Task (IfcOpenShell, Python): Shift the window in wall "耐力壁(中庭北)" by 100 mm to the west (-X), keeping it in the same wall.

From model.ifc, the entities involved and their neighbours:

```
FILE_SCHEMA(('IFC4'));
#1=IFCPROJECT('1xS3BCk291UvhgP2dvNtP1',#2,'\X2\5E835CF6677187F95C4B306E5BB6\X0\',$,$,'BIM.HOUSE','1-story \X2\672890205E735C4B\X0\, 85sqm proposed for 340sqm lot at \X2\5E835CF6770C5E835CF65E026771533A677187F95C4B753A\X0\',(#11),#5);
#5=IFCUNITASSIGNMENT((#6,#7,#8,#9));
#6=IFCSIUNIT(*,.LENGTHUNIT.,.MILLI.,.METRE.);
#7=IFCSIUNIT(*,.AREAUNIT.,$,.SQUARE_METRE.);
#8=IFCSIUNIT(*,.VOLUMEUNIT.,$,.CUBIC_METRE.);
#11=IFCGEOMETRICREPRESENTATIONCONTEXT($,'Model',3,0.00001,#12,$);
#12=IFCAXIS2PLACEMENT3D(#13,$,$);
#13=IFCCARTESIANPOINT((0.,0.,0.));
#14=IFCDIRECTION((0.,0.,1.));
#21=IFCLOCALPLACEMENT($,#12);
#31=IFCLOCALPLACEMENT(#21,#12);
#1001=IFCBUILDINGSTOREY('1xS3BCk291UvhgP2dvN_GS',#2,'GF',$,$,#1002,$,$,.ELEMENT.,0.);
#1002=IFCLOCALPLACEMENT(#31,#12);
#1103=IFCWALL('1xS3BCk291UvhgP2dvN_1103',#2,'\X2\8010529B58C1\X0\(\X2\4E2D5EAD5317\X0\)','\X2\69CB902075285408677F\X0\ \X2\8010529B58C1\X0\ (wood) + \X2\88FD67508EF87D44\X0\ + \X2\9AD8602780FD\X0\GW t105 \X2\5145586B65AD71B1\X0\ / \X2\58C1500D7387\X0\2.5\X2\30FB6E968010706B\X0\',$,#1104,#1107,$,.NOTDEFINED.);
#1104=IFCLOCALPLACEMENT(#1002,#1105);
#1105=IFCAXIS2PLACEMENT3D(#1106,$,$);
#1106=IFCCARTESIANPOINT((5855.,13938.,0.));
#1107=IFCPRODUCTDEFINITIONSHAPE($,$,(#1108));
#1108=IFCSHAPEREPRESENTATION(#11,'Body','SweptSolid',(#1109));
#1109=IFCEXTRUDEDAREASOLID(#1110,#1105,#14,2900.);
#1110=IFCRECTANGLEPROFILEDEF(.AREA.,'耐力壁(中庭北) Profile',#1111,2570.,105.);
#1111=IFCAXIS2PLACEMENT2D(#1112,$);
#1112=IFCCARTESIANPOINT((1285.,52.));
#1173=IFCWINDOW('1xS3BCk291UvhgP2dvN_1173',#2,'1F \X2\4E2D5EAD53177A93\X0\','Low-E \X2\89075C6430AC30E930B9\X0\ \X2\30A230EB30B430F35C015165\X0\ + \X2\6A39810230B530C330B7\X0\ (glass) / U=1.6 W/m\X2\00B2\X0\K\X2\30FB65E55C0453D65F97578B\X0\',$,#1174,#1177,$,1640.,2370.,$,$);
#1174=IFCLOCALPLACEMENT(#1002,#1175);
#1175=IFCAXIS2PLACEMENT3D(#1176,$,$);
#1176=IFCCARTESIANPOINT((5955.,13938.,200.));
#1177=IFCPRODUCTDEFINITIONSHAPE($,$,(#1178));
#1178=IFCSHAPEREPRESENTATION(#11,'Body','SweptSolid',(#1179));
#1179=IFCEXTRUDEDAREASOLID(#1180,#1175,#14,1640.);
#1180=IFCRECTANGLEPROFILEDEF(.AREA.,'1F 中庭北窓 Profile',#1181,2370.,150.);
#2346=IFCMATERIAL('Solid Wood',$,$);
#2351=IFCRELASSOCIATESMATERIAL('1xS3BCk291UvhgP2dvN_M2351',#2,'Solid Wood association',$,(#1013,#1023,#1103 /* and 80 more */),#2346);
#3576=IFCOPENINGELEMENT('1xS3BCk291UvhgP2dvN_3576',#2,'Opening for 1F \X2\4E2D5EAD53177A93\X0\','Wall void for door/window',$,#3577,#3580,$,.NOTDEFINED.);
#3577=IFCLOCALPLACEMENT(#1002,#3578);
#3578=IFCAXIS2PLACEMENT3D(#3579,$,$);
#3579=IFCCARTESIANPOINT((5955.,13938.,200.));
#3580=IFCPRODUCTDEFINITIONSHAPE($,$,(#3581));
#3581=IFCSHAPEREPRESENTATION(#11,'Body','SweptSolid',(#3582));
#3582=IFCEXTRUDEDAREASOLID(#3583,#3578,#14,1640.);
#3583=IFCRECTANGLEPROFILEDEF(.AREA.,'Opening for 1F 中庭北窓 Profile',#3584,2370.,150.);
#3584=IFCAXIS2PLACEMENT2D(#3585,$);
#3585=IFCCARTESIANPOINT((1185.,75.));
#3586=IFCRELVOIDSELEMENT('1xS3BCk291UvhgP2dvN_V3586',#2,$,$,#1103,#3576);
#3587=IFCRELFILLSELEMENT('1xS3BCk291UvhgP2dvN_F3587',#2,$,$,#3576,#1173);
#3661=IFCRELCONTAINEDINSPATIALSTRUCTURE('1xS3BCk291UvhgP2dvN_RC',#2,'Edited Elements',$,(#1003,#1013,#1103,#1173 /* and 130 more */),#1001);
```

```python
import ifcopenshell
import ifcopenshell.api.geometry
import ifcopenshell.util.placement

model = ifcopenshell.open("model.ifc")

window = model.by_guid("1xS3BCk291UvhgP2dvN_1173")
opening = window.FillsVoids[0].RelatingOpeningElement
wall = opening.VoidsElements[0].RelatingBuildingElement

wall_matrix = ifcopenshell.util.placement.get_local_placement(wall.ObjectPlacement)
shift = wall_matrix[:3, 0] * -100.0
before = ifcopenshell.util.placement.get_local_placement(window.ObjectPlacement)[:3, 3].copy()

# The window is not placed relative to its opening, so move both.
for product in (opening, window):
    matrix = ifcopenshell.util.placement.get_local_placement(product.ObjectPlacement)
    matrix[:3, 3] += shift
    ifcopenshell.api.geometry.edit_object_placement(model, product=product, matrix=matrix, is_si=False)

after = ifcopenshell.util.placement.get_local_placement(window.ObjectPlacement)[:3, 3]
print("window moved by", (after - before).round(3) + 0.0)

model.write("model-out.ifc")
```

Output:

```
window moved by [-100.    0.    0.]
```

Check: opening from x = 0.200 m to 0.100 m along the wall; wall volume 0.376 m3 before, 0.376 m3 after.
